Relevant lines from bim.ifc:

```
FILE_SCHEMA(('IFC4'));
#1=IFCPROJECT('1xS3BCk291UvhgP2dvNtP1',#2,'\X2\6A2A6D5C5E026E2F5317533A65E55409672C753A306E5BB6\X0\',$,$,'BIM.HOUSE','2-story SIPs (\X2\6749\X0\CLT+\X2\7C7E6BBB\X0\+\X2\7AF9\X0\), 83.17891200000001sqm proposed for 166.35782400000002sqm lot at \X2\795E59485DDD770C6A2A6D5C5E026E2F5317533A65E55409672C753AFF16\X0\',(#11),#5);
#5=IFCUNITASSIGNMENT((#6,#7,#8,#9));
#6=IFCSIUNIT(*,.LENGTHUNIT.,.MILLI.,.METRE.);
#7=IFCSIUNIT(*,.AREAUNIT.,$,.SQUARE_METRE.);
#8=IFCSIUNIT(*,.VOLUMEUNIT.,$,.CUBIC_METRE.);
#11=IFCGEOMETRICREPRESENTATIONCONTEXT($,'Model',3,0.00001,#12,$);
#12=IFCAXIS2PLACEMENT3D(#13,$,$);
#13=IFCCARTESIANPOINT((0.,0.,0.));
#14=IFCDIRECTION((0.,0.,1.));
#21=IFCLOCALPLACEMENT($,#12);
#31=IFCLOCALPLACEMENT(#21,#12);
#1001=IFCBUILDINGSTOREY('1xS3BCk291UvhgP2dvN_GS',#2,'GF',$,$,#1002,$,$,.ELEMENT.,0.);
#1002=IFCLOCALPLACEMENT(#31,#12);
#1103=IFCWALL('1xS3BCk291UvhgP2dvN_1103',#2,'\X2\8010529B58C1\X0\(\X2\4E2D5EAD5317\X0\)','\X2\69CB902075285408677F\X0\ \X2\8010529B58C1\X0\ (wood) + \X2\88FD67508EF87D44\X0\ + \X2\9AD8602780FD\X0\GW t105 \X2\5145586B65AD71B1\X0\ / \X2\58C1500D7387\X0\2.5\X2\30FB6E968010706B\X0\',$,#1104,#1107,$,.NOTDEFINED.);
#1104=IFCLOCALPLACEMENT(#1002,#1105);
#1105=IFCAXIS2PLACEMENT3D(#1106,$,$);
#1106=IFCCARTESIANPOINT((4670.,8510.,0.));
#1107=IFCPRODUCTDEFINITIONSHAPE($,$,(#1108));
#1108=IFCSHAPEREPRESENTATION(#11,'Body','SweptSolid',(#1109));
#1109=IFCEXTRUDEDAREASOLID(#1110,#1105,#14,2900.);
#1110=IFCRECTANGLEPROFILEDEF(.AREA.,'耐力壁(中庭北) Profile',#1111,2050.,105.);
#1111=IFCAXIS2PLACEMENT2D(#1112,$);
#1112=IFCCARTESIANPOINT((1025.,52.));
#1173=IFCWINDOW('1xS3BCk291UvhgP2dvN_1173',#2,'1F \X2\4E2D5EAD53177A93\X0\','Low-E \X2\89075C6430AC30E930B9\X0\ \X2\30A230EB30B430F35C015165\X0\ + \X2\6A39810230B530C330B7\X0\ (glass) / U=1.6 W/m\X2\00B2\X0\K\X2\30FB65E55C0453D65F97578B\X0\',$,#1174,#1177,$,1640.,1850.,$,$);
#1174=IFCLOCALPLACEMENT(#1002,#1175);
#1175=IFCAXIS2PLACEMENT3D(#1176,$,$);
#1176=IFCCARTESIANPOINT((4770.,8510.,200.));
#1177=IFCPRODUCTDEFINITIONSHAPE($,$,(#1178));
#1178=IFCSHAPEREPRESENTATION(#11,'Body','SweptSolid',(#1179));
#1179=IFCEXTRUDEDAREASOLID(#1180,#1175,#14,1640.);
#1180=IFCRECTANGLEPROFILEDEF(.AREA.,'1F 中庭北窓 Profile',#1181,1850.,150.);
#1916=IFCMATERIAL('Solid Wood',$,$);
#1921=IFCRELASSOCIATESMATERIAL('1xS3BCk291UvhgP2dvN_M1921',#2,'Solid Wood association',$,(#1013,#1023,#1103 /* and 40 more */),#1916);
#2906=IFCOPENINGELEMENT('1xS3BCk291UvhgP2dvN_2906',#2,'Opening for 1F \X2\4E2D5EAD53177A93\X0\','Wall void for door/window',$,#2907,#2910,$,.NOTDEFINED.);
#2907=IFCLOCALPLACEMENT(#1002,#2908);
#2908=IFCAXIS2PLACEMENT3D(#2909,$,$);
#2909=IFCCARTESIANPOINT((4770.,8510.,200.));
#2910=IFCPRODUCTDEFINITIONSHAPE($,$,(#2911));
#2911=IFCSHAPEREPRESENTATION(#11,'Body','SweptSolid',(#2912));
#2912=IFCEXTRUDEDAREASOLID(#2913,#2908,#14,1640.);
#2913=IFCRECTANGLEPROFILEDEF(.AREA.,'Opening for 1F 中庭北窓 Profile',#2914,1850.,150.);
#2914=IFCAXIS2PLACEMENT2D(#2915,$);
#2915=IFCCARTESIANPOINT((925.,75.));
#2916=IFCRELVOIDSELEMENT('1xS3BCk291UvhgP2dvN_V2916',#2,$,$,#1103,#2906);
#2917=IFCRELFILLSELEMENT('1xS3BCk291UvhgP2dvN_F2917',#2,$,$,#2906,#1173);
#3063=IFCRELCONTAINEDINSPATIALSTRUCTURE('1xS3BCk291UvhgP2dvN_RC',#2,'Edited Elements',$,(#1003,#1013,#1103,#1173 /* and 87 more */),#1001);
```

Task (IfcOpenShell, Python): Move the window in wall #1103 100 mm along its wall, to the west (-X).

```python
import ifcopenshell
import ifcopenshell.api.geometry
import ifcopenshell.util.placement
import ifcopenshell.util.unit

model = ifcopenshell.open("bim.ifc")
unit_scale = ifcopenshell.util.unit.calculate_unit_scale(model)

window = model.by_id(1173)
opening = window.FillsVoids[0].RelatingOpeningElement
wall = opening.VoidsElements[0].RelatingBuildingElement

wall_matrix = ifcopenshell.util.placement.get_local_placement(wall.ObjectPlacement)
shift = wall_matrix[:3, 0] * -0.1 / unit_scale
before = ifcopenshell.util.placement.get_local_placement(window.ObjectPlacement)[:3, 3].copy()

# The window is not placed relative to its opening, so move both.
for product in (opening, window):
    matrix = ifcopenshell.util.placement.get_local_placement(product.ObjectPlacement)
    matrix[:3, 3] += shift
    ifcopenshell.api.geometry.edit_object_placement(model, product=product, matrix=matrix, is_si=False)

after = ifcopenshell.util.placement.get_local_placement(window.ObjectPlacement)[:3, 3]
print("window moved by", (after - before).round(3) + 0.0)

model.write("bim_updated.ifc")
```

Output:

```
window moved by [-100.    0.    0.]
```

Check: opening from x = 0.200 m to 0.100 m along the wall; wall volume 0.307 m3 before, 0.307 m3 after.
